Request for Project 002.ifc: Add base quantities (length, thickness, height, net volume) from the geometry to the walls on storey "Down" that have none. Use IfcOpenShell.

First a look at what the model holds.

```python
import ifcopenshell
import ifcopenshell.util.element
import ifcopenshell.util.unit

model = ifcopenshell.open("Project 002.ifc")
print(model.schema)
for unit_type in ("LENGTHUNIT", "AREAUNIT", "VOLUMEUNIT"):
    print(unit_type, ifcopenshell.util.unit.calculate_unit_scale(model, unit_type))
storey = next(s for s in model.by_type("IfcBuildingStorey") if s.Name == "Down")
walls = [e for e in ifcopenshell.util.element.get_decomposition(storey) if e.is_a("IfcWall")]
for e in sorted(walls, key=lambda e: e.id()):
    print(e.id(), e.is_a(), e.Name, list(ifcopenshell.util.element.get_psets(e, qtos_only=True)), sep=" | ")
```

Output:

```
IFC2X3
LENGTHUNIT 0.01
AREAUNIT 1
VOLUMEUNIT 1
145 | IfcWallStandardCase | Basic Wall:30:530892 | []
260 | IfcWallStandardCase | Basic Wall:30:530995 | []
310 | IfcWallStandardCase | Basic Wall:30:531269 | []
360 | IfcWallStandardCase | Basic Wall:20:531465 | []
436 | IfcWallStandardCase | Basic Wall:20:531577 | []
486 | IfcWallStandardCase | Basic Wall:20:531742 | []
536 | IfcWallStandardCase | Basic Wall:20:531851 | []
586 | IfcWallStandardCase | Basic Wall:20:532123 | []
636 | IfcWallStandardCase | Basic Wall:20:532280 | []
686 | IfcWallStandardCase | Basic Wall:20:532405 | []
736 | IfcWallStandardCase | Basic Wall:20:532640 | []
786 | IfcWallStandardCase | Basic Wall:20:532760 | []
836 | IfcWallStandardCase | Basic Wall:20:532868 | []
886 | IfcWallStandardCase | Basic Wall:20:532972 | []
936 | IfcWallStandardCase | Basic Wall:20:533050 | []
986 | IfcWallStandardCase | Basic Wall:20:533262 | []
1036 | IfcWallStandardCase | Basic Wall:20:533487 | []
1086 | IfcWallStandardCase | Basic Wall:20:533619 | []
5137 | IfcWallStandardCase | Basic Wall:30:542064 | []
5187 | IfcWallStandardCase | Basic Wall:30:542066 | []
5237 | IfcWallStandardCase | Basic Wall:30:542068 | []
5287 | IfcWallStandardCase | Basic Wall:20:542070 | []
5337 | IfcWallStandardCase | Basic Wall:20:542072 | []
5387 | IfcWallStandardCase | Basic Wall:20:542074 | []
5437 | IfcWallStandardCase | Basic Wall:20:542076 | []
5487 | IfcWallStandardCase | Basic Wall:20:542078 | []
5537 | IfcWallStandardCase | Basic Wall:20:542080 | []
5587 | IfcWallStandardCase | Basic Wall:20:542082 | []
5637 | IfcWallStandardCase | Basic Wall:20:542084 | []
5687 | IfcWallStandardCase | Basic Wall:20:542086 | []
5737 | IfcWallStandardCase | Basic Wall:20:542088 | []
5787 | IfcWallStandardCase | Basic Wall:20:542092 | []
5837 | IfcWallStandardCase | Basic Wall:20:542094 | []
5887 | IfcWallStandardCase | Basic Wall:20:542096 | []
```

```python
import ifcopenshell
import ifcopenshell.api.pset
import ifcopenshell.geom
import ifcopenshell.util.element
import ifcopenshell.util.shape
import ifcopenshell.util.unit

model = ifcopenshell.open("Project 002.ifc")
unit_scale = ifcopenshell.util.unit.calculate_unit_scale(model)
volume_scale = ifcopenshell.util.unit.calculate_unit_scale(model, "VOLUMEUNIT")
settings = ifcopenshell.geom.settings()

storey = next(s for s in model.by_type("IfcBuildingStorey") if s.Name == "Down")
walls = [e for e in ifcopenshell.util.element.get_decomposition(storey) if e.is_a("IfcWall")]

for e in sorted(walls, key=lambda e: e.id()):
    if ifcopenshell.util.element.get_psets(e, qtos_only=True, should_inherit=False):
        continue
    # Geometry comes back in metres, in the element's own axes.
    shape = ifcopenshell.geom.create_shape(settings, e)
    values = {
        "Length": ifcopenshell.util.shape.get_x(shape.geometry) / unit_scale,
        "Width": ifcopenshell.util.shape.get_y(shape.geometry) / unit_scale,
        "Height": ifcopenshell.util.shape.get_z(shape.geometry) / unit_scale,
        "NetVolume": ifcopenshell.util.shape.get_volume(shape.geometry) / volume_scale,
    }
    qto = ifcopenshell.api.pset.add_qto(model, product=e, name="BaseQuantities")
    ifcopenshell.api.pset.edit_qto(model, qto=qto, properties=values)
    print(e.id(), {k: round(v, 3) for k, v in values.items()})

model.write("Project 002_rev.ifc")
```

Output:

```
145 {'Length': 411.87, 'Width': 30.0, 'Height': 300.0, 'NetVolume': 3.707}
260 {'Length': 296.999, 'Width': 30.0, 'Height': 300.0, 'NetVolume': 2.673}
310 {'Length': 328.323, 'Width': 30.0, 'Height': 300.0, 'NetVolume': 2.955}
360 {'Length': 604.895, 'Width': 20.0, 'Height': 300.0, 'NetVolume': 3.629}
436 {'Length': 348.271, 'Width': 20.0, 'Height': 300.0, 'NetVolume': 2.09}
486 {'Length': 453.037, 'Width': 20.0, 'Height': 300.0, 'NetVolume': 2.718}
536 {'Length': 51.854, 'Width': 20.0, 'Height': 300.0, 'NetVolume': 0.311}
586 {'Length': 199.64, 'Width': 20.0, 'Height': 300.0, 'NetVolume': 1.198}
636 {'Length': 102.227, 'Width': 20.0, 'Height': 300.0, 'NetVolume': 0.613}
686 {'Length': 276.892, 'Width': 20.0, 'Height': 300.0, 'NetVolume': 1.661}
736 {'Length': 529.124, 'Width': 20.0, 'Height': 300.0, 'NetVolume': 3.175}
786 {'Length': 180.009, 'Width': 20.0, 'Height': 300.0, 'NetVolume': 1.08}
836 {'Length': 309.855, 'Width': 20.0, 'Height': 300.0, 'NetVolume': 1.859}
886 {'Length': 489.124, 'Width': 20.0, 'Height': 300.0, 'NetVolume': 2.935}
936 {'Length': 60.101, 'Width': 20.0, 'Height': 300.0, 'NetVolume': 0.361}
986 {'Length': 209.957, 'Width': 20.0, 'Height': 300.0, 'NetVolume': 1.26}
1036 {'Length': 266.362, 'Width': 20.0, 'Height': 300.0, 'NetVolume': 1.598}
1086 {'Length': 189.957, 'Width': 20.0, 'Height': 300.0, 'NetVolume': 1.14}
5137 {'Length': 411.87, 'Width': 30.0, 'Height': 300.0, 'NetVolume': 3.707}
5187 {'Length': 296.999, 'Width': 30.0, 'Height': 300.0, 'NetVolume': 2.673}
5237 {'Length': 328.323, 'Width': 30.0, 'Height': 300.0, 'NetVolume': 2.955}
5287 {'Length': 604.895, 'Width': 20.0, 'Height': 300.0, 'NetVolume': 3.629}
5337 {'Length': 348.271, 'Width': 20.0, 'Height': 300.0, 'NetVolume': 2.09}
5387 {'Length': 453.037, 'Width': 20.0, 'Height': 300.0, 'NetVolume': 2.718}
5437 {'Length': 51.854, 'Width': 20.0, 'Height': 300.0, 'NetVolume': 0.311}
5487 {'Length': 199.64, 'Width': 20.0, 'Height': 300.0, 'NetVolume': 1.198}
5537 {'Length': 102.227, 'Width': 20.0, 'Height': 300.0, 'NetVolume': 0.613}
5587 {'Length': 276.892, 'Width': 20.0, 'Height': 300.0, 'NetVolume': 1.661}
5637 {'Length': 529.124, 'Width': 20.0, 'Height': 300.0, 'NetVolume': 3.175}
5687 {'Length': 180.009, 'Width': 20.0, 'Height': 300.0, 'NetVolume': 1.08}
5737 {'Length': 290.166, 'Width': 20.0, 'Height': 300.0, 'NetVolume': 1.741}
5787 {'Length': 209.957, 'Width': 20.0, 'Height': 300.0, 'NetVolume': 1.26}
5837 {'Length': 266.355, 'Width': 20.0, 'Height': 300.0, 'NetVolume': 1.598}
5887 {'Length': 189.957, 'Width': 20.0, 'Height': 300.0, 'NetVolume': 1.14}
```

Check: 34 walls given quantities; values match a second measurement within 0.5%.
